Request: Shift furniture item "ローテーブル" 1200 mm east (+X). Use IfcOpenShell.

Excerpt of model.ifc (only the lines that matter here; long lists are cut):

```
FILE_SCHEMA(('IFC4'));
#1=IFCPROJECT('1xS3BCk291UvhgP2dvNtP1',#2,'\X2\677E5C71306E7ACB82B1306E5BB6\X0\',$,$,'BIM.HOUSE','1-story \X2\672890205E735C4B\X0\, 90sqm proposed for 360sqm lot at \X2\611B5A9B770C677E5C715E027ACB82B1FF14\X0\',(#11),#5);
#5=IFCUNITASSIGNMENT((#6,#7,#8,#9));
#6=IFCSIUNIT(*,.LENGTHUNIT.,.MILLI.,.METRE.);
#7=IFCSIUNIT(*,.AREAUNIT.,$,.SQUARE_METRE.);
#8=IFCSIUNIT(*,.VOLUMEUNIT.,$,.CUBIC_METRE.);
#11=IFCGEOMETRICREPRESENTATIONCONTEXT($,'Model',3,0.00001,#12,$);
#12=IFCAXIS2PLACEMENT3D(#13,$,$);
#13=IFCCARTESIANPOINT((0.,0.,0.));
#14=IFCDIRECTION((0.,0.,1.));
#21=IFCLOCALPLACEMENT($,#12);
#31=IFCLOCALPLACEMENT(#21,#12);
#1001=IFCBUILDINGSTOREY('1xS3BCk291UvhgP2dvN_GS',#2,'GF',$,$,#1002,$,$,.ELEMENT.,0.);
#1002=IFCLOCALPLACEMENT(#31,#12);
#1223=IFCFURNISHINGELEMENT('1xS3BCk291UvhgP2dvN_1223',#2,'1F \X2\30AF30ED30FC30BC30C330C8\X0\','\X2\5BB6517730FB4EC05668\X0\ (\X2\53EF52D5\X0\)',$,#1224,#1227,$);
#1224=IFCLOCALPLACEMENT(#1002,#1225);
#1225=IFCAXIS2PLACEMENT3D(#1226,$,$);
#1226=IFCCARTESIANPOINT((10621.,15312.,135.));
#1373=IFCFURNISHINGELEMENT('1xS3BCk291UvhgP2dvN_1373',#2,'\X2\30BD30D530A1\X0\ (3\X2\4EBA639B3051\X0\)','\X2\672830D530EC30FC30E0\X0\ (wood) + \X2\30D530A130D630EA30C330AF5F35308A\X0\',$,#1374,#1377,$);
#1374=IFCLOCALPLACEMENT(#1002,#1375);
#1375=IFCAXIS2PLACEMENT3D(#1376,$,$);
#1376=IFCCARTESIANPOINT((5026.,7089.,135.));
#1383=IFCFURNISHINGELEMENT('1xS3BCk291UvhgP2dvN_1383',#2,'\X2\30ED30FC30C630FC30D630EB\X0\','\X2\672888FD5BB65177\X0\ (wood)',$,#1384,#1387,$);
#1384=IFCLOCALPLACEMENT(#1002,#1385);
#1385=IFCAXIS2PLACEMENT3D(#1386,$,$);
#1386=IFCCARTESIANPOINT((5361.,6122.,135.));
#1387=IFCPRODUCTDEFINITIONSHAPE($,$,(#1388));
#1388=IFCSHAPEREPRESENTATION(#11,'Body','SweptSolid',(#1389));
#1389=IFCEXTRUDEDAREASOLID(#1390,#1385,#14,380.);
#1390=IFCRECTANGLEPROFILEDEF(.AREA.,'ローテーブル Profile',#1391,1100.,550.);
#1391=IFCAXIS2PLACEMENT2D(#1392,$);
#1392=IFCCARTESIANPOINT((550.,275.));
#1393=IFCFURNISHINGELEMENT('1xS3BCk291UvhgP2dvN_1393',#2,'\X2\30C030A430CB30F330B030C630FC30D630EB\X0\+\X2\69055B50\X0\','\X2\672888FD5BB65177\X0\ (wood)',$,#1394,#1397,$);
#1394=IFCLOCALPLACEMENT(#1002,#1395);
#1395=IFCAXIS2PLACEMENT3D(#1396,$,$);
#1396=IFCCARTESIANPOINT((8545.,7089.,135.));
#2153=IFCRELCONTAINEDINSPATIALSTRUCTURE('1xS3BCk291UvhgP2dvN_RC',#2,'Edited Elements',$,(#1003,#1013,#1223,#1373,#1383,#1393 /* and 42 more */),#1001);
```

```python
import ifcopenshell
import ifcopenshell.api.geometry
import ifcopenshell.util.placement

model = ifcopenshell.open("model.ifc")

item = model.by_id(1383)
matrix = ifcopenshell.util.placement.get_local_placement(item.ObjectPlacement)
matrix[0, 3] += 1200.0
ifcopenshell.api.geometry.edit_object_placement(model, product=item, matrix=matrix, is_si=False)

print(ifcopenshell.util.placement.get_local_placement(item.ObjectPlacement).round(3) + 0.0)

model.write("model_updated.ifc")
```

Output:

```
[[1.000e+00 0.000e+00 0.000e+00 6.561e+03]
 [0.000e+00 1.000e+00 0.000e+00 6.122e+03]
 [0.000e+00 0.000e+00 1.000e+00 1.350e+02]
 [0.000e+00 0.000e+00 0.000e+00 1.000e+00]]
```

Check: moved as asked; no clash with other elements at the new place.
